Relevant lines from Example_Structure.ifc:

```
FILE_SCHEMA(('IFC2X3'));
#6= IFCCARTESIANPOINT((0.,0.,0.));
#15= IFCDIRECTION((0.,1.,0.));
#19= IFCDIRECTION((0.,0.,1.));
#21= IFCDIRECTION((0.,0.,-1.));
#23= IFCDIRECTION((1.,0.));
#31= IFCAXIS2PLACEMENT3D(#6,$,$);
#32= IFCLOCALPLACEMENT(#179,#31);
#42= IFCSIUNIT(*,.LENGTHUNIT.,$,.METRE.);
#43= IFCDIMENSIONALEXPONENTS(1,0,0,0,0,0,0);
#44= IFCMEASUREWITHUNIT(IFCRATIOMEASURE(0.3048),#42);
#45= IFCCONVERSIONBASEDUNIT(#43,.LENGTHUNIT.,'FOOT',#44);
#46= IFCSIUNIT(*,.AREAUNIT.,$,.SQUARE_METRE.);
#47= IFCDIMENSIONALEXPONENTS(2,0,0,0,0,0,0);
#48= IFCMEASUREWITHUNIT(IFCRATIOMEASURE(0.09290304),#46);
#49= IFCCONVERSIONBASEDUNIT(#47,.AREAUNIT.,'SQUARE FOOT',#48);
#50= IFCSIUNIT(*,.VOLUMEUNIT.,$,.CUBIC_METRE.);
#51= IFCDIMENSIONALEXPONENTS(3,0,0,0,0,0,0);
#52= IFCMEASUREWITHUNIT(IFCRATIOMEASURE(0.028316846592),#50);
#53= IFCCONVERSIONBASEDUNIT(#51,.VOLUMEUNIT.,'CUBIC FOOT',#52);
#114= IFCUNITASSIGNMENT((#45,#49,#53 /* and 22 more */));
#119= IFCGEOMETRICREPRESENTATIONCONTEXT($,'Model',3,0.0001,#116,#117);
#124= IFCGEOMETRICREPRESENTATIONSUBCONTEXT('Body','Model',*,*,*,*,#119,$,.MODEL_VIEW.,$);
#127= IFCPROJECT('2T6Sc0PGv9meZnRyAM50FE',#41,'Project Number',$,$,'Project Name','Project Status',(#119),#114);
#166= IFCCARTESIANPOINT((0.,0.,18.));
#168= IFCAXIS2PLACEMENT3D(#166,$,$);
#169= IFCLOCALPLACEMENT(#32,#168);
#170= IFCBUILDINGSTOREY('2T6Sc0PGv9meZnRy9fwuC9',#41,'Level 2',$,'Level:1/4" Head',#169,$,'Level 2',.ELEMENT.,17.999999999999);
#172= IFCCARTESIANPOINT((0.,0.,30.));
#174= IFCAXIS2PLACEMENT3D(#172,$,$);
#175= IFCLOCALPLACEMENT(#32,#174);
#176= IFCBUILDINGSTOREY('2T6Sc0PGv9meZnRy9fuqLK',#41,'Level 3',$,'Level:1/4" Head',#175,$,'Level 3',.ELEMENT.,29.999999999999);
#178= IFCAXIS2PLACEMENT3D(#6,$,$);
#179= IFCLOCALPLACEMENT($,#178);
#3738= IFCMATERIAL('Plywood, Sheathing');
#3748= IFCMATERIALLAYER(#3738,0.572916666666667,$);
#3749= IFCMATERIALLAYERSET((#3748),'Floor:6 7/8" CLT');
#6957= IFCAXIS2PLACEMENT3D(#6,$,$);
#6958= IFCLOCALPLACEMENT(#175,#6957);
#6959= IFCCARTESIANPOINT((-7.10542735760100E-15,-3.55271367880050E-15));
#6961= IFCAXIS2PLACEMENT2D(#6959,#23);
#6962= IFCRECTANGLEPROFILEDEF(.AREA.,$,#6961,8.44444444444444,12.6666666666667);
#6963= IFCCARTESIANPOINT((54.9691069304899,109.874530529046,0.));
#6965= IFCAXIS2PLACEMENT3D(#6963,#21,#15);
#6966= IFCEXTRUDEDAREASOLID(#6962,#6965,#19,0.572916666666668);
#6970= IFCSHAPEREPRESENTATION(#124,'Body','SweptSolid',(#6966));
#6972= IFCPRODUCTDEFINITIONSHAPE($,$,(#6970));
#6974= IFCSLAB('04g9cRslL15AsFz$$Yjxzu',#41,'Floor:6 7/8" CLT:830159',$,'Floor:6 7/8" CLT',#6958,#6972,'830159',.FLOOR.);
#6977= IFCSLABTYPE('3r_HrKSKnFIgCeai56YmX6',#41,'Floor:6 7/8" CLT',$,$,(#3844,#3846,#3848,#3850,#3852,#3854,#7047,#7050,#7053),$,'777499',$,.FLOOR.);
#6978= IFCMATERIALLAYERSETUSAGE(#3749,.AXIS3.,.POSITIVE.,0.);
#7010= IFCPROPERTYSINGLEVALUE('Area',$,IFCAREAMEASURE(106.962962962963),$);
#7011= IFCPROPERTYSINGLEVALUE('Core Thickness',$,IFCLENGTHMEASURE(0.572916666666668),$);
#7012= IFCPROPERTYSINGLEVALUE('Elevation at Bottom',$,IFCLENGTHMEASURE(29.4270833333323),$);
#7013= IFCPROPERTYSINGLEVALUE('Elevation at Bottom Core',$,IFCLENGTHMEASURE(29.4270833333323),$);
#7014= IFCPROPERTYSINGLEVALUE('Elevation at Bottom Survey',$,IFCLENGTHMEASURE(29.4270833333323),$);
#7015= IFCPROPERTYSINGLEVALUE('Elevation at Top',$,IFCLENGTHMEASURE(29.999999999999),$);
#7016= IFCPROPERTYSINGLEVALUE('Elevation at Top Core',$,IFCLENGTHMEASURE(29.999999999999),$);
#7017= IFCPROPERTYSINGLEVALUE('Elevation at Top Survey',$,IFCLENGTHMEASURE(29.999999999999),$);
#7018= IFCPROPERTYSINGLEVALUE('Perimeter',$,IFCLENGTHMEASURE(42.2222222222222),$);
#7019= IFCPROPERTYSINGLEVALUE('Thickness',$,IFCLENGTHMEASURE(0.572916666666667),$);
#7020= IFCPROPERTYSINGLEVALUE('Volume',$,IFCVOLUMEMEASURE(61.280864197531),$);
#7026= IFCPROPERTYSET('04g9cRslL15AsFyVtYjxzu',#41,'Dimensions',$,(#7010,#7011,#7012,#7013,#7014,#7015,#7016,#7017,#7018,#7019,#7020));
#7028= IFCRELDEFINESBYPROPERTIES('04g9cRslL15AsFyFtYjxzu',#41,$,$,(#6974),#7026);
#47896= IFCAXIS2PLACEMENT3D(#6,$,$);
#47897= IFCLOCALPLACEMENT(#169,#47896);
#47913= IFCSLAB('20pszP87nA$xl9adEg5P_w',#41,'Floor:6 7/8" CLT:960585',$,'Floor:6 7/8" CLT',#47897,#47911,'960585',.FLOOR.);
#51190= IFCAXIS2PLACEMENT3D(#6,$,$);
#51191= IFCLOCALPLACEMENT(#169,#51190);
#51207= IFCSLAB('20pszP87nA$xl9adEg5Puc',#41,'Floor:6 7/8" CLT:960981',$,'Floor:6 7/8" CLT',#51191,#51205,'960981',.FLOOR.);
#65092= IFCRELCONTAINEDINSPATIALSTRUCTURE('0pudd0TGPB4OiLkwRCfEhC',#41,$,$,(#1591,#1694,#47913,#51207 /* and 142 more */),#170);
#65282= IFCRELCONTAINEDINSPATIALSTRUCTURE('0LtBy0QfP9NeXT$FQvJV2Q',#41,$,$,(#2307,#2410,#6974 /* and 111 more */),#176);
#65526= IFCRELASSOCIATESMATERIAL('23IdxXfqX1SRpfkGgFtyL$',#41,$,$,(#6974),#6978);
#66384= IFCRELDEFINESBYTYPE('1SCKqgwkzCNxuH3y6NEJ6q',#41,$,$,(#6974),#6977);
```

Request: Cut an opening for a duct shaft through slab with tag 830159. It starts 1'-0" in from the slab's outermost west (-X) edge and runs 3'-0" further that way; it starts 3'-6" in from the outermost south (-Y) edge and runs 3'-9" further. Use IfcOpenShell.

```python
import numpy as np
import ifcopenshell
import ifcopenshell.api.feature
import ifcopenshell.api.geometry
import ifcopenshell.api.pset
import ifcopenshell.api.root
import ifcopenshell.geom
import ifcopenshell.util.element
import ifcopenshell.util.placement
import ifcopenshell.util.representation
import ifcopenshell.util.shape
import ifcopenshell.util.unit

model = ifcopenshell.open("Example_Structure.ifc")
unit_scale = ifcopenshell.util.unit.calculate_unit_scale(model)
area_scale = ifcopenshell.util.unit.calculate_unit_scale(model, "AREAUNIT")
volume_scale = ifcopenshell.util.unit.calculate_unit_scale(model, "VOLUMEUNIT")
settings = ifcopenshell.geom.settings()


def volume(element):
    """Net volume in cubic metres, openings subtracted."""
    shape = ifcopenshell.geom.create_shape(settings, element)
    return ifcopenshell.util.shape.get_volume(shape.geometry)


slab = model.by_guid("04g9cRslL15AsFz$$Yjxzu")
before = volume(slab)

# Extent in the slab's own axes, in metres. The edges named are its -X and -Y sides.
slab_shape = ifcopenshell.geom.create_shape(settings, slab)
vertices = ifcopenshell.util.shape.get_vertices(slab_shape.geometry)
x_min, y_min, bottom = vertices.min(axis=0)
top = vertices[:, 2].max()

opening = ifcopenshell.api.root.create_entity(model, ifc_class="IfcOpeningElement", name="Duct shaft opening")
context = ifcopenshell.util.representation.get_context(model, "Model", "Body", "MODEL_VIEW")
width, depth = 0.9144, 1.143
outline = [(0.0, 0.0), (width, 0.0), (width, depth), (0.0, depth), (0.0, 0.0)]
# Overshoot both faces by 50 mm so the cut is clean.
shape = ifcopenshell.api.geometry.add_slab_representation(
    model, context=context, depth=top - bottom + 0.1, polyline=outline
)
ifcopenshell.api.geometry.assign_representation(model, product=opening, representation=shape)

matrix = ifcopenshell.util.placement.get_local_placement(slab.ObjectPlacement)
matrix[:, 3] = matrix @ np.append(np.array([x_min + 0.3048, y_min + 1.0668, bottom - 0.05]) / unit_scale, 1.0)
ifcopenshell.api.geometry.edit_object_placement(model, product=opening, matrix=matrix, is_si=False)
ifcopenshell.api.feature.add_feature(model, feature=opening, element=slab)

after = volume(slab)

# Update the slab's stored quantities.
pset = model.by_id(ifcopenshell.util.element.get_pset(slab, "Dimensions", should_inherit=False)["id"])
ifcopenshell.api.pset.edit_pset(model, pset=pset, properties={
    "Area": model.create_entity("IfcAreaMeasure", after / (top - bottom) / area_scale),
    "Volume": model.create_entity("IfcVolumeMeasure", after / volume_scale),
})

print(f"slab volume {before:.3f} -> {after:.3f} m3")

model.write("Example_Structure-out.ifc")
```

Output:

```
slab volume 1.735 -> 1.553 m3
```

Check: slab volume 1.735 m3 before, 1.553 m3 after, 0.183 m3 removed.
